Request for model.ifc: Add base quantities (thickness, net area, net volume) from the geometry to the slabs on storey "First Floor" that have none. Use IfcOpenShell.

First a look at what the model holds.

```python
import ifcopenshell
import ifcopenshell.util.element
import ifcopenshell.util.unit

model = ifcopenshell.open("model.ifc")
print(model.schema)
for unit_type in ("LENGTHUNIT", "AREAUNIT", "VOLUMEUNIT"):
    print(unit_type, ifcopenshell.util.unit.calculate_unit_scale(model, unit_type))
storey = next(s for s in model.by_type("IfcBuildingStorey") if s.Name == "First Floor")
slabs = [e for e in ifcopenshell.util.element.get_decomposition(storey) if e.is_a("IfcSlab")]
for e in sorted(slabs, key=lambda e: e.id()):
    print(e.id(), e.is_a(), e.Name, list(ifcopenshell.util.element.get_psets(e, qtos_only=True)), sep=" | ")
```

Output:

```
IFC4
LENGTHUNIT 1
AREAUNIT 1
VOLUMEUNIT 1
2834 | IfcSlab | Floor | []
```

```python
import ifcopenshell
import ifcopenshell.api.pset
import ifcopenshell.geom
import ifcopenshell.util.element
import ifcopenshell.util.shape
import ifcopenshell.util.unit

model = ifcopenshell.open("model.ifc")
unit_scale = ifcopenshell.util.unit.calculate_unit_scale(model)
area_scale = ifcopenshell.util.unit.calculate_unit_scale(model, "AREAUNIT")
volume_scale = ifcopenshell.util.unit.calculate_unit_scale(model, "VOLUMEUNIT")
settings = ifcopenshell.geom.settings()

storey = next(s for s in model.by_type("IfcBuildingStorey") if s.Name == "First Floor")
slabs = [e for e in ifcopenshell.util.element.get_decomposition(storey) if e.is_a("IfcSlab")]

for e in sorted(slabs, key=lambda e: e.id()):
    if ifcopenshell.util.element.get_psets(e, qtos_only=True, should_inherit=False):
        continue
    # Geometry comes back in metres, in the element's own axes.
    shape = ifcopenshell.geom.create_shape(settings, e)
    values = {
        "Width": ifcopenshell.util.shape.get_z(shape.geometry) / unit_scale,
        "NetArea": ifcopenshell.util.shape.get_footprint_area(shape.geometry) / area_scale,
        "NetVolume": ifcopenshell.util.shape.get_volume(shape.geometry) / volume_scale,
    }
    qto = ifcopenshell.api.pset.add_qto(model, product=e, name="Qto_SlabBaseQuantities")
    ifcopenshell.api.pset.edit_qto(model, qto=qto, properties=values)
    print(e.id(), {k: round(v, 3) for k, v in values.items()})

model.write("model-out.ifc")
```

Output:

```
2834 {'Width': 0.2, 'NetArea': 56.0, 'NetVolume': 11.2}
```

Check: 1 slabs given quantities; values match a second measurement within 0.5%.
